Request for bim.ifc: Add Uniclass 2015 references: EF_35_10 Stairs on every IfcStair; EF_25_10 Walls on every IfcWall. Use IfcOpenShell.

First a look at what the model holds.

```python
import ifcopenshell

model = ifcopenshell.open("bim.ifc")
print(model.schema)
print("classifications:", [c.Name for c in model.by_type("IfcClassification")])
for ifc_class in ("IfcDoor", "IfcRoof", "IfcStair", "IfcWall", "IfcWindow"):
    print(ifc_class, len(model.by_type(ifc_class)))
```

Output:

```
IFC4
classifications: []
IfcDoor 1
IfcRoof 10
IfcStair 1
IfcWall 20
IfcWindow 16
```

```python
import ifcopenshell
import ifcopenshell.api.classification

model = ifcopenshell.open("bim.ifc")

system = ifcopenshell.api.classification.add_classification(model, classification="Uniclass 2015")

codes = {
    "IfcStair": ("EF_35_10", "Stairs"),
    "IfcWall": ("EF_25_10", "Walls"),
}
for ifc_class, (code, name) in codes.items():
    products = model.by_type(ifc_class)
    ifcopenshell.api.classification.add_reference(
        model, products=products, classification=system, identification=code, name=name
    )
    print(code, len(products))

model.write("bim-out.ifc")
```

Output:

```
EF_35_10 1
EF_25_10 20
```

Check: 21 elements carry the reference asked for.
